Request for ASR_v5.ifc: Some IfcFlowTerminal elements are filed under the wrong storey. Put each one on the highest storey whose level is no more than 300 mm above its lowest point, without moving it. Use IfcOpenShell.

First a look at what the model holds.

```python
import ifcopenshell
import ifcopenshell.util.element
import ifcopenshell.util.placement

model = ifcopenshell.open("ASR_v5.ifc")
print(model.schema)
for storey in model.by_type("IfcBuildingStorey"):
    level = ifcopenshell.util.placement.get_storey_elevation(storey)
    count = sum(e.is_a("IfcFlowTerminal") for e in ifcopenshell.util.element.get_contained(storey))
    print(storey.id(), storey.Name, round(level, 3), count, sep=" | ")
```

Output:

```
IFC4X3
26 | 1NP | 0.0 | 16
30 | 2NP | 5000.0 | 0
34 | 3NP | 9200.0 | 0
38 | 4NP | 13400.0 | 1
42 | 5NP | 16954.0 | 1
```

```python
import ifcopenshell
import ifcopenshell.api.spatial
import ifcopenshell.geom
import ifcopenshell.util.element
import ifcopenshell.util.placement
import ifcopenshell.util.shape
import ifcopenshell.util.unit

model = ifcopenshell.open("ASR_v5.ifc")
unit_scale = ifcopenshell.util.unit.calculate_unit_scale(model)
settings = ifcopenshell.geom.settings()

levels = sorted(
    ((ifcopenshell.util.placement.get_storey_elevation(s) * unit_scale, s) for s in model.by_type("IfcBuildingStorey")),
    key=lambda pair: pair[0],
)

for e in model.by_type("IfcFlowTerminal"):
    current = e.ContainedInStructure[0].RelatingStructure if e.ContainedInStructure else None
    if current is None or not current.is_a("IfcBuildingStorey"):
        continue
    shape = ifcopenshell.geom.create_shape(settings, e)
    bottom = ifcopenshell.util.shape.get_shape_bottom_elevation(shape, shape.geometry)
    below = [s for level, s in levels if level <= bottom + 0.3]
    storey = below[-1] if below else levels[0][1]
    if storey != current:
        # assign_container keeps the world position.
        ifcopenshell.api.spatial.assign_container(model, products=[e], relating_structure=storey)
        print(e.id(), current.Name, "->", storey.Name)

model.write("ASR_v5-out.ifc")
```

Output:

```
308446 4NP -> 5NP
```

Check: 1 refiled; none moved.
